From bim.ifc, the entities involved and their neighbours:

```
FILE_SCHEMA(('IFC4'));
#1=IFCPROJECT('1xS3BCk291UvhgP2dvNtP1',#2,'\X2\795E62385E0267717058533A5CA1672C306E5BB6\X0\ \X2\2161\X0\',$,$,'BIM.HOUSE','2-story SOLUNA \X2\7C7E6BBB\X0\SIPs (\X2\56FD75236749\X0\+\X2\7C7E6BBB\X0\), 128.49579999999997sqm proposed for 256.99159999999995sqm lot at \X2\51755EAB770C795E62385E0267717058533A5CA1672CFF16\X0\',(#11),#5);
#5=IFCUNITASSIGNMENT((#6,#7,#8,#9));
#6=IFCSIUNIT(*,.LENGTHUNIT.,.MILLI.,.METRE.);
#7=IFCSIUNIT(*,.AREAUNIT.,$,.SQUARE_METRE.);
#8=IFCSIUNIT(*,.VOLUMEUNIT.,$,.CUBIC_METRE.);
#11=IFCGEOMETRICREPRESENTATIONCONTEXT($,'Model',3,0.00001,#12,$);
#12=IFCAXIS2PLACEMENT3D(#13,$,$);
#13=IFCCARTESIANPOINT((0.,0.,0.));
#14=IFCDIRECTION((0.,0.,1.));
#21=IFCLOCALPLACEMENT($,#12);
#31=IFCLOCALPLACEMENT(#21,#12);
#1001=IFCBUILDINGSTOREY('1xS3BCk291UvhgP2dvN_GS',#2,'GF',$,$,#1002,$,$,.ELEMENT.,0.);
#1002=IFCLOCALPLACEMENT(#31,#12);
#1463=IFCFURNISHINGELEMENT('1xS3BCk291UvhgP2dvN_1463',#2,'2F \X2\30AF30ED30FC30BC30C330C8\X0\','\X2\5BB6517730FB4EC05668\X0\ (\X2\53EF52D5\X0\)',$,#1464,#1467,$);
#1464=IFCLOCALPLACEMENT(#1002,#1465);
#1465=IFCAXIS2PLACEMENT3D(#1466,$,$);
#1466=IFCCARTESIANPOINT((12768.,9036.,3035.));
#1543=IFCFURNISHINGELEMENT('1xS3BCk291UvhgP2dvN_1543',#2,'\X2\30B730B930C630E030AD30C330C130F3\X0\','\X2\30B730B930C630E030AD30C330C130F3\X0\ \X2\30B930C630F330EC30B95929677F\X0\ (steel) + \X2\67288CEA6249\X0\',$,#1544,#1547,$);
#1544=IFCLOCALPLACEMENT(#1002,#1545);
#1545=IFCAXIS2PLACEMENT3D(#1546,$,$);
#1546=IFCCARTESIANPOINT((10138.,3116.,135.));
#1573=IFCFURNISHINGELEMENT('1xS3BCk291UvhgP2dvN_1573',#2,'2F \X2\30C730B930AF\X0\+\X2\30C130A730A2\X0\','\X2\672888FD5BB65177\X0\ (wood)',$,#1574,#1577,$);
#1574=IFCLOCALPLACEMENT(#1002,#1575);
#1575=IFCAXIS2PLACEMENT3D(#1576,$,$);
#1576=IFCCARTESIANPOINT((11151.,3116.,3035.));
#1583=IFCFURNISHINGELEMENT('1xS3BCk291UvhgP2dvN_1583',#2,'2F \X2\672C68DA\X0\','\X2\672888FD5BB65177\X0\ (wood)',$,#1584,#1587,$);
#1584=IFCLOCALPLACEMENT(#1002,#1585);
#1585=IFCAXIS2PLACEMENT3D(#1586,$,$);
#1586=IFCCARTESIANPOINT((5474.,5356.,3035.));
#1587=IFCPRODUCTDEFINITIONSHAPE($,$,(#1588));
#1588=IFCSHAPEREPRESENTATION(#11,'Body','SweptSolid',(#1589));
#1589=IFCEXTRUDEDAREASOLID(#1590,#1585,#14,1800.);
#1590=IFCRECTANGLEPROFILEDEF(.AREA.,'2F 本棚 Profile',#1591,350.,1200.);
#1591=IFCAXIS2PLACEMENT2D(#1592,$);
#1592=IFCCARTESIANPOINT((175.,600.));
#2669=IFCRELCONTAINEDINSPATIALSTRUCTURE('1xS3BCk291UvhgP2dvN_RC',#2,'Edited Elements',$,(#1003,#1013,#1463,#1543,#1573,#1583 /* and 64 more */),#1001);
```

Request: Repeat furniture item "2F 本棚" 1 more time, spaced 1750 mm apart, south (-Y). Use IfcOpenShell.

```python
import numpy as np
import ifcopenshell
import ifcopenshell.api.geometry
import ifcopenshell.api.root
import ifcopenshell.util.element
import ifcopenshell.util.placement

model = ifcopenshell.open("bim.ifc")


def reuse_history(source, copy):
    """copy_class also copies each property set's owner history, people and application; keep the originals."""
    for rel in copy.IsDefinedBy:
        if rel.is_a("IfcRelDefinesByProperties") and (history := rel.RelatingPropertyDefinition.OwnerHistory):
            rel.RelatingPropertyDefinition.OwnerHistory = source.OwnerHistory
            ifcopenshell.util.element.remove_deep2(model, history)


source = model.by_guid("1xS3BCk291UvhgP2dvN_1583")
base = ifcopenshell.util.placement.get_local_placement(source.ObjectPlacement)
step = np.array([0.0, -1.0, 0.0]) * 1750.0

for i in range(1, 2):
    copy = ifcopenshell.api.root.copy_class(model, product=source)
    copy.Representation = ifcopenshell.util.element.copy_deep(
        model, source.Representation, exclude=["IfcGeometricRepresentationContext", "IfcRepresentationMap"]
    )
    reuse_history(source, copy)
    matrix = base.copy()
    matrix[:3, 3] += i * step
    print("added at", matrix[:3, 3].round(3) + 0.0)
    ifcopenshell.api.geometry.edit_object_placement(model, product=copy, matrix=matrix, is_si=False)

model.write("bim_rev.ifc")
```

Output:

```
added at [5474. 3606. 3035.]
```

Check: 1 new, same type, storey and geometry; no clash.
